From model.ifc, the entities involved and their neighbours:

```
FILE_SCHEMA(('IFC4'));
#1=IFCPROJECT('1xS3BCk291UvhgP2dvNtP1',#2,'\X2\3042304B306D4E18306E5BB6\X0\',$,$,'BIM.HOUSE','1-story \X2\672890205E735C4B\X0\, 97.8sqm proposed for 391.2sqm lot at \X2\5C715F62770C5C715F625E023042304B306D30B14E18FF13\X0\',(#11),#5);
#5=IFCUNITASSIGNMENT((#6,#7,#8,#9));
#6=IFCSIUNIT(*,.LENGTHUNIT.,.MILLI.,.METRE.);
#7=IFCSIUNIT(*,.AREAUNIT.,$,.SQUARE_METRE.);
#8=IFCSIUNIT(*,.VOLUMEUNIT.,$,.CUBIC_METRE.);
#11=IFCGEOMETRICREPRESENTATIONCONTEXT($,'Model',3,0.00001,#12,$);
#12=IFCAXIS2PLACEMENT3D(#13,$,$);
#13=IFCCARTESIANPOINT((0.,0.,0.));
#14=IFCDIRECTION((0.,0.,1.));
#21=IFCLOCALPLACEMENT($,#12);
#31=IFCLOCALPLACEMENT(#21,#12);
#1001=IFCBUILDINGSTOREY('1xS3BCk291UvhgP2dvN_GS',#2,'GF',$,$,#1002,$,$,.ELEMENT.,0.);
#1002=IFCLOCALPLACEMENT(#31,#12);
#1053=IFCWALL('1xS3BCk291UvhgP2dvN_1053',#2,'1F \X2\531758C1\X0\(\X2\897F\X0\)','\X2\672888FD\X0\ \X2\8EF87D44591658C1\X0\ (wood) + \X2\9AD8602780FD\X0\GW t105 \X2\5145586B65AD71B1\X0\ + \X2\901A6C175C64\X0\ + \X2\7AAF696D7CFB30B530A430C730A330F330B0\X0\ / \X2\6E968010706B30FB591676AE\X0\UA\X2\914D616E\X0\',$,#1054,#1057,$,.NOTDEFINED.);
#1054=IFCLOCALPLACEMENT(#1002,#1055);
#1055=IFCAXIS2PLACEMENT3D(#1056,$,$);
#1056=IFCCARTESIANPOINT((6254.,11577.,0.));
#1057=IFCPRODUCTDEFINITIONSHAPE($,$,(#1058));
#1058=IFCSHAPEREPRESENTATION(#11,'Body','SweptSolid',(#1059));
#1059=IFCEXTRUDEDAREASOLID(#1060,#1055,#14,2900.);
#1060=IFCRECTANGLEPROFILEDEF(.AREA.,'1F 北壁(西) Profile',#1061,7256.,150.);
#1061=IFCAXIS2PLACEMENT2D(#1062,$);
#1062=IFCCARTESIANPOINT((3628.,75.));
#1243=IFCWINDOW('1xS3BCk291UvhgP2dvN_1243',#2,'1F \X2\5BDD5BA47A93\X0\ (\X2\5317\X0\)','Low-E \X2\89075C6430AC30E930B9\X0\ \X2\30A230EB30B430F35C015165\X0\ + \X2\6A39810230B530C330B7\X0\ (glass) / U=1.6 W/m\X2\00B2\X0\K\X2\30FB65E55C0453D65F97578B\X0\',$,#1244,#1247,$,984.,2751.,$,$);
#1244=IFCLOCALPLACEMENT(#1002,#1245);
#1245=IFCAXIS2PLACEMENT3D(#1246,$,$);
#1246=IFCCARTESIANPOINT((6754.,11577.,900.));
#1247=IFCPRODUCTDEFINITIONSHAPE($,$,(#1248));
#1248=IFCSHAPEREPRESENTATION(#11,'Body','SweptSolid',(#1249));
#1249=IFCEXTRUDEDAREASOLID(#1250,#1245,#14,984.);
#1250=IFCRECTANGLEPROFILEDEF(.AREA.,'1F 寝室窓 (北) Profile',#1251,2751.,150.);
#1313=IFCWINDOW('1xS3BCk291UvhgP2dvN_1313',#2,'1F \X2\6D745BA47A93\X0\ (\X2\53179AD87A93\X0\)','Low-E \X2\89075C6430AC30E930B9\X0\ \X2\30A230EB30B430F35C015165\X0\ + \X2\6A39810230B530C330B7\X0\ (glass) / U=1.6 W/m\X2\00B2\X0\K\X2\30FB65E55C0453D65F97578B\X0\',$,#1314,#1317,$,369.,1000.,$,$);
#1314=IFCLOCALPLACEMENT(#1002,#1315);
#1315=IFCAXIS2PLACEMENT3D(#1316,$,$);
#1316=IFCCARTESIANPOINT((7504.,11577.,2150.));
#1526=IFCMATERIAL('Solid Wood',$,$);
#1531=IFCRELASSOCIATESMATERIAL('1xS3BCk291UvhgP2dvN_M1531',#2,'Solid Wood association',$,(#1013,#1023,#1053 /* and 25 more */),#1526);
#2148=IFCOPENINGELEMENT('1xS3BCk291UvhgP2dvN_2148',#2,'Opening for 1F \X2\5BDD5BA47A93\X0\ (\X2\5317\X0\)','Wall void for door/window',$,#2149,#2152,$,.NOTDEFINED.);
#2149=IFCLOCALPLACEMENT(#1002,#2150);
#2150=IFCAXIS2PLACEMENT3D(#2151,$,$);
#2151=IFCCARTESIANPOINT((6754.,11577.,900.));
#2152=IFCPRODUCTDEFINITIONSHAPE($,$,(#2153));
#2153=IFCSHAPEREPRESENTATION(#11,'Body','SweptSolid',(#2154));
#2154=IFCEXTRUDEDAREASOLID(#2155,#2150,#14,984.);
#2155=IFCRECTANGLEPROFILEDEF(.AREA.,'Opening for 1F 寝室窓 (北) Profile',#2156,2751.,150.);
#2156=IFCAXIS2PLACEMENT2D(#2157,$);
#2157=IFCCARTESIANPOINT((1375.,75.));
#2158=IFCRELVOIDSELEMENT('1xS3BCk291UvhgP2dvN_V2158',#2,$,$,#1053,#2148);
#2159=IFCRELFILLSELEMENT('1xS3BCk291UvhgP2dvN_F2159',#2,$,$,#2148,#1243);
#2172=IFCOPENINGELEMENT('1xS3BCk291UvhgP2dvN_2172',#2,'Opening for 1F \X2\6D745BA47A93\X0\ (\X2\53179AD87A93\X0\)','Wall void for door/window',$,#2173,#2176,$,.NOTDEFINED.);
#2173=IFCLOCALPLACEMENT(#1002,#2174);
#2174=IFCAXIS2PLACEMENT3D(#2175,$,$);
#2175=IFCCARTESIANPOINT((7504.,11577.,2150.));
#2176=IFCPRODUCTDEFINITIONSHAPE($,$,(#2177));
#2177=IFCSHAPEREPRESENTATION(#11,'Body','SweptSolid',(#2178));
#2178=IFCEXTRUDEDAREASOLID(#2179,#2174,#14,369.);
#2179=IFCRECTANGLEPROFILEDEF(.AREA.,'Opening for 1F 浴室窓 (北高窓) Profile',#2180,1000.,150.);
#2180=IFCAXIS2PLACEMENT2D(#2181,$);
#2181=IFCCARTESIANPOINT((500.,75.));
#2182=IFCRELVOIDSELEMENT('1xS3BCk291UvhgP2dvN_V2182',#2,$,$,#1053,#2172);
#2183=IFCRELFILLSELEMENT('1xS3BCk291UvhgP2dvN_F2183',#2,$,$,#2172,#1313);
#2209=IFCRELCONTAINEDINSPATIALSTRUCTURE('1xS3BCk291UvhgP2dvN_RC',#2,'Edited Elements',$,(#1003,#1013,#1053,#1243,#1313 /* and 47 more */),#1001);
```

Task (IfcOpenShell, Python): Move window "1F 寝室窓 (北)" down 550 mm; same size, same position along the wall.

```python
import numpy as np
import ifcopenshell
import ifcopenshell.api.geometry
import ifcopenshell.util.placement
import ifcopenshell.util.unit

model = ifcopenshell.open("model.ifc")
unit_scale = ifcopenshell.util.unit.calculate_unit_scale(model)

window = model.by_guid("1xS3BCk291UvhgP2dvN_1243")
opening = window.FillsVoids[0].RelatingOpeningElement
dz = -550.0

shift = np.array([0.0, 0.0, dz])
# The window is not placed relative to its opening, so move both.
for product in (opening, window):
    matrix = ifcopenshell.util.placement.get_local_placement(product.ObjectPlacement)
    matrix[:3, 3] += shift
    ifcopenshell.api.geometry.edit_object_placement(model, product=product, matrix=matrix, is_si=False)

print(f"moved by {dz * unit_scale:+.3f} m")

model.write("model_v2.ifc")
```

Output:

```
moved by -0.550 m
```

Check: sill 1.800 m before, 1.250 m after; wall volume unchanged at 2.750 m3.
